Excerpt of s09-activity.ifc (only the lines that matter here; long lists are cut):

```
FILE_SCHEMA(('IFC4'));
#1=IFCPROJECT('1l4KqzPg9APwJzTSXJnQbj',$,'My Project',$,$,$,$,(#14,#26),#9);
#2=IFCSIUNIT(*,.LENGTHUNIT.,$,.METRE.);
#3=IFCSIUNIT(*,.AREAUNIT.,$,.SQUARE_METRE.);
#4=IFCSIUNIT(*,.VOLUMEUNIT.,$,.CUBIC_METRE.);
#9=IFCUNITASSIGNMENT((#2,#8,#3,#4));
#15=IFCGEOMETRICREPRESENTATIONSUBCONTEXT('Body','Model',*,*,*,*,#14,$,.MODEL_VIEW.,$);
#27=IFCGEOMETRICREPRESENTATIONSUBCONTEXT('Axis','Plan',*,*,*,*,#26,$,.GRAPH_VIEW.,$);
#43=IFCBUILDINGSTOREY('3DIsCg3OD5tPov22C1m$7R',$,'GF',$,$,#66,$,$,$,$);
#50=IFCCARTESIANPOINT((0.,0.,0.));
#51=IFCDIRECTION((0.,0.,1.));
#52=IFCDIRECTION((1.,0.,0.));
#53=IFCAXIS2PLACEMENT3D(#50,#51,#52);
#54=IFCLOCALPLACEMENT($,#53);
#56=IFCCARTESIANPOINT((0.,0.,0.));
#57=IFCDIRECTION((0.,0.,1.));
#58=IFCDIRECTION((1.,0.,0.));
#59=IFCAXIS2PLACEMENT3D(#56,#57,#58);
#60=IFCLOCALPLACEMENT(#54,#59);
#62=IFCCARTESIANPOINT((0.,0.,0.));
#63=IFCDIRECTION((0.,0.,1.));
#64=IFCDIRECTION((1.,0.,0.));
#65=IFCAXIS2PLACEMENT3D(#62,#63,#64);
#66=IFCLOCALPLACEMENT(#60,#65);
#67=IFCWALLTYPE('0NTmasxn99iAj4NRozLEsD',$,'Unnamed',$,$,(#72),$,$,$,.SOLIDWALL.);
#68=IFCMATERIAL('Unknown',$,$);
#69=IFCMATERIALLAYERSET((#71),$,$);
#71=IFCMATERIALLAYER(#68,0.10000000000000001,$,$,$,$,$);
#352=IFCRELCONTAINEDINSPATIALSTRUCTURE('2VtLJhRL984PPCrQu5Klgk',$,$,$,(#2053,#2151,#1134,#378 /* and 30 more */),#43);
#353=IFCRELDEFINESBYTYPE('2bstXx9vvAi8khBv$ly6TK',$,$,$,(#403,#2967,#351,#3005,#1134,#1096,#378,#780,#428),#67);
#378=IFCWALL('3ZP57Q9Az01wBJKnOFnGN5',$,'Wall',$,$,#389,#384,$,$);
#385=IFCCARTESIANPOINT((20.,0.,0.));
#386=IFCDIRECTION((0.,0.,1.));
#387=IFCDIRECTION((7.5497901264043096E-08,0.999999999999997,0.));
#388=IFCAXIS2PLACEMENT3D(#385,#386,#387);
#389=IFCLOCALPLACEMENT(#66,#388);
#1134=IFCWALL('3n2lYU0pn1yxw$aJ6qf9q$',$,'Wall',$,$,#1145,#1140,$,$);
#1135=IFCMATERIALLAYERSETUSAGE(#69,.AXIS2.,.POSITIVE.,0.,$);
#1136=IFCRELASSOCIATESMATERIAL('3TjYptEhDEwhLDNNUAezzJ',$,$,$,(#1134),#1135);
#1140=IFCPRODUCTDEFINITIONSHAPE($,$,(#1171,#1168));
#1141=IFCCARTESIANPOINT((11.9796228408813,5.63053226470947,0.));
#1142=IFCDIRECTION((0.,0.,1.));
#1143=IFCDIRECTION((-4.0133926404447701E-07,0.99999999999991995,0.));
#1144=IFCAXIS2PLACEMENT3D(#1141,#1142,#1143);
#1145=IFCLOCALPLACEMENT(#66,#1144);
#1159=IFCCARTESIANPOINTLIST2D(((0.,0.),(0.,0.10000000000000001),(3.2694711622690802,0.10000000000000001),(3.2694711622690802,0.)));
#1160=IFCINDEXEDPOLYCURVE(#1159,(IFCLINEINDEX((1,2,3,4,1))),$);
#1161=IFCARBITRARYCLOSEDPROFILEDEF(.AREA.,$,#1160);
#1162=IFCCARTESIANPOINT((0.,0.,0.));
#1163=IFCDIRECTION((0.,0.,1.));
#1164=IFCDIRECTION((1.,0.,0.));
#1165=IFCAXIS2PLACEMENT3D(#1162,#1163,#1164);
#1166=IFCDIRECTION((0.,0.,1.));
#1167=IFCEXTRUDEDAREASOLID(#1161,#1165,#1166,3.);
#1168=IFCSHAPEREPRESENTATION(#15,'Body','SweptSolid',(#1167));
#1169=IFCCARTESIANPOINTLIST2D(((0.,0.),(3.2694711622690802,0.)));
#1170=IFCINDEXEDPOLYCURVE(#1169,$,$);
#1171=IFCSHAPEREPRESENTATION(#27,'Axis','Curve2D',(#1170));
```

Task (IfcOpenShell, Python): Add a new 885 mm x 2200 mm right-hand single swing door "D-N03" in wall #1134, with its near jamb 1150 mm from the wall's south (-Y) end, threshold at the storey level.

```python
import numpy as np
import ifcopenshell
import ifcopenshell.api.feature
import ifcopenshell.api.geometry
import ifcopenshell.api.root
import ifcopenshell.api.spatial
import ifcopenshell.geom
import ifcopenshell.util.element
import ifcopenshell.util.placement
import ifcopenshell.util.representation
import ifcopenshell.util.shape
import ifcopenshell.util.unit

model = ifcopenshell.open("s09-activity.ifc")
unit_scale = ifcopenshell.util.unit.calculate_unit_scale(model)
settings = ifcopenshell.geom.settings()


def volume(element):
    """Net volume in cubic metres, openings subtracted."""
    shape = ifcopenshell.geom.create_shape(settings, element)
    return ifcopenshell.util.shape.get_volume(shape.geometry)


wall = model.by_guid("3n2lYU0pn1yxw$aJ6qf9q$")
storey = ifcopenshell.util.element.get_container(wall, ifc_class="IfcBuildingStorey")
context = ifcopenshell.util.representation.get_context(model, "Model", "Body", "MODEL_VIEW")
before = volume(wall)

width, height, from_end, sill = 0.885, 2.2, 1.15, 0.0  # metres

# The wall runs along its own X axis, and the end named is its -X end.
wall_shape = ifcopenshell.geom.create_shape(settings, wall)
x, y, z = ifcopenshell.util.shape.get_vertices(wall_shape.geometry).T
start = x.min() + from_end
face, thickness = float(y.min()), float(y.max() - y.min())
wall_matrix = ifcopenshell.util.placement.get_local_placement(wall.ObjectPlacement)
level = ifcopenshell.util.placement.get_local_placement(storey.ObjectPlacement)[2, 3]


def in_wall(x, y):
    """Placement at x, y metres in the wall's axes, at sill height."""
    matrix = wall_matrix.copy()
    matrix[:, 3] = wall_matrix @ np.array([x / unit_scale, y / unit_scale, 0.0, 1.0])
    matrix[2, 3] = level + sill / unit_scale
    return matrix


# Opening: a box that overshoots both wall faces by 50 mm.
opening = ifcopenshell.api.root.create_entity(model, ifc_class="IfcOpeningElement", predefined_type="OPENING")
box = ifcopenshell.api.geometry.add_wall_representation(
    model, context=context, length=width, height=height, thickness=thickness + 0.1
)
ifcopenshell.api.geometry.assign_representation(model, product=opening, representation=box)
ifcopenshell.api.geometry.edit_object_placement(model, product=opening, matrix=in_wall(start, face - 0.05), is_si=False)
ifcopenshell.api.feature.add_feature(model, feature=opening, element=wall)

door = ifcopenshell.api.root.create_entity(model, ifc_class="IfcDoor", name="D-N03", predefined_type="DOOR")
door.OverallWidth, door.OverallHeight = width / unit_scale, height / unit_scale
door.OperationType = "SINGLE_SWING_RIGHT"
body = ifcopenshell.api.geometry.add_door_representation(
    model,
    context=context,
    overall_width=door.OverallWidth,
    overall_height=door.OverallHeight,
    operation_type="SINGLE_SWING_RIGHT",
    lining_properties={"LiningDepth": thickness / unit_scale, "ThresholdDepth": thickness / unit_scale},
)
ifcopenshell.api.geometry.assign_representation(model, product=door, representation=body)
ifcopenshell.api.spatial.assign_container(model, products=[door], relating_structure=storey)
ifcopenshell.api.feature.add_filling(model, opening=opening, element=door)

# The lining spans the wall, so the door starts at the wall face.
ifcopenshell.api.geometry.edit_object_placement(model, product=door, matrix=in_wall(start, face), is_si=False)

after = volume(wall)

print(f"wall volume {before:.3f} -> {after:.3f} m3")

model.write("s09-activity_edited.ifc")
```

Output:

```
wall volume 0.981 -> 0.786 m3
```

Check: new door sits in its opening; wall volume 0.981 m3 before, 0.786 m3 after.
